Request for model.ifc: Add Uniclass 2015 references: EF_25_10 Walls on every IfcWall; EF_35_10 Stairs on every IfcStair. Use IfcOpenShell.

First a look at what the model holds.

```python
import ifcopenshell

model = ifcopenshell.open("model.ifc")
print(model.schema)
print("classifications:", [c.Name for c in model.by_type("IfcClassification")])
for ifc_class in ("IfcDoor", "IfcRoof", "IfcStair", "IfcWall", "IfcWindow"):
    print(ifc_class, len(model.by_type(ifc_class)))
```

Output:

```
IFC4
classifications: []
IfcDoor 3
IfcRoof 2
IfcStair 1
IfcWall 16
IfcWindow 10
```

```python
import ifcopenshell
import ifcopenshell.api.classification

model = ifcopenshell.open("model.ifc")

system = ifcopenshell.api.classification.add_classification(model, classification="Uniclass 2015")

codes = {
    "IfcWall": ("EF_25_10", "Walls"),
    "IfcStair": ("EF_35_10", "Stairs"),
}
for ifc_class, (code, name) in codes.items():
    products = model.by_type(ifc_class)
    ifcopenshell.api.classification.add_reference(
        model, products=products, classification=system, identification=code, name=name
    )
    print(code, len(products))

model.write("model_edited.ifc")
```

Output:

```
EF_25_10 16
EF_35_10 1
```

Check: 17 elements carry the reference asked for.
